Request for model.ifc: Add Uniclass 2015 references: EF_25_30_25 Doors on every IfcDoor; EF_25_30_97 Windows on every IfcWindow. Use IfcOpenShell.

First a look at what the model holds.

```python
import ifcopenshell

model = ifcopenshell.open("model.ifc")
print(model.schema)
print("classifications:", [c.Name for c in model.by_type("IfcClassification")])
for ifc_class in ("IfcDoor", "IfcRoof", "IfcStair", "IfcWall", "IfcWindow"):
    print(ifc_class, len(model.by_type(ifc_class)))
```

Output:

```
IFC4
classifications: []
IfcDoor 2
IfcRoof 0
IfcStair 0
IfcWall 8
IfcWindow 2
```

```python
import ifcopenshell
import ifcopenshell.api.classification

model = ifcopenshell.open("model.ifc")

system = ifcopenshell.api.classification.add_classification(model, classification="Uniclass 2015")

codes = {
    "IfcDoor": ("EF_25_30_25", "Doors"),
    "IfcWindow": ("EF_25_30_97", "Windows"),
}
for ifc_class, (code, name) in codes.items():
    products = model.by_type(ifc_class)
    ifcopenshell.api.classification.add_reference(
        model, products=products, classification=system, identification=code, name=name
    )
    print(code, len(products))

model.write("model-out.ifc")
```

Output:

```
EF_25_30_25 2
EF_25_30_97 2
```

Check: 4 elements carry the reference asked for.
